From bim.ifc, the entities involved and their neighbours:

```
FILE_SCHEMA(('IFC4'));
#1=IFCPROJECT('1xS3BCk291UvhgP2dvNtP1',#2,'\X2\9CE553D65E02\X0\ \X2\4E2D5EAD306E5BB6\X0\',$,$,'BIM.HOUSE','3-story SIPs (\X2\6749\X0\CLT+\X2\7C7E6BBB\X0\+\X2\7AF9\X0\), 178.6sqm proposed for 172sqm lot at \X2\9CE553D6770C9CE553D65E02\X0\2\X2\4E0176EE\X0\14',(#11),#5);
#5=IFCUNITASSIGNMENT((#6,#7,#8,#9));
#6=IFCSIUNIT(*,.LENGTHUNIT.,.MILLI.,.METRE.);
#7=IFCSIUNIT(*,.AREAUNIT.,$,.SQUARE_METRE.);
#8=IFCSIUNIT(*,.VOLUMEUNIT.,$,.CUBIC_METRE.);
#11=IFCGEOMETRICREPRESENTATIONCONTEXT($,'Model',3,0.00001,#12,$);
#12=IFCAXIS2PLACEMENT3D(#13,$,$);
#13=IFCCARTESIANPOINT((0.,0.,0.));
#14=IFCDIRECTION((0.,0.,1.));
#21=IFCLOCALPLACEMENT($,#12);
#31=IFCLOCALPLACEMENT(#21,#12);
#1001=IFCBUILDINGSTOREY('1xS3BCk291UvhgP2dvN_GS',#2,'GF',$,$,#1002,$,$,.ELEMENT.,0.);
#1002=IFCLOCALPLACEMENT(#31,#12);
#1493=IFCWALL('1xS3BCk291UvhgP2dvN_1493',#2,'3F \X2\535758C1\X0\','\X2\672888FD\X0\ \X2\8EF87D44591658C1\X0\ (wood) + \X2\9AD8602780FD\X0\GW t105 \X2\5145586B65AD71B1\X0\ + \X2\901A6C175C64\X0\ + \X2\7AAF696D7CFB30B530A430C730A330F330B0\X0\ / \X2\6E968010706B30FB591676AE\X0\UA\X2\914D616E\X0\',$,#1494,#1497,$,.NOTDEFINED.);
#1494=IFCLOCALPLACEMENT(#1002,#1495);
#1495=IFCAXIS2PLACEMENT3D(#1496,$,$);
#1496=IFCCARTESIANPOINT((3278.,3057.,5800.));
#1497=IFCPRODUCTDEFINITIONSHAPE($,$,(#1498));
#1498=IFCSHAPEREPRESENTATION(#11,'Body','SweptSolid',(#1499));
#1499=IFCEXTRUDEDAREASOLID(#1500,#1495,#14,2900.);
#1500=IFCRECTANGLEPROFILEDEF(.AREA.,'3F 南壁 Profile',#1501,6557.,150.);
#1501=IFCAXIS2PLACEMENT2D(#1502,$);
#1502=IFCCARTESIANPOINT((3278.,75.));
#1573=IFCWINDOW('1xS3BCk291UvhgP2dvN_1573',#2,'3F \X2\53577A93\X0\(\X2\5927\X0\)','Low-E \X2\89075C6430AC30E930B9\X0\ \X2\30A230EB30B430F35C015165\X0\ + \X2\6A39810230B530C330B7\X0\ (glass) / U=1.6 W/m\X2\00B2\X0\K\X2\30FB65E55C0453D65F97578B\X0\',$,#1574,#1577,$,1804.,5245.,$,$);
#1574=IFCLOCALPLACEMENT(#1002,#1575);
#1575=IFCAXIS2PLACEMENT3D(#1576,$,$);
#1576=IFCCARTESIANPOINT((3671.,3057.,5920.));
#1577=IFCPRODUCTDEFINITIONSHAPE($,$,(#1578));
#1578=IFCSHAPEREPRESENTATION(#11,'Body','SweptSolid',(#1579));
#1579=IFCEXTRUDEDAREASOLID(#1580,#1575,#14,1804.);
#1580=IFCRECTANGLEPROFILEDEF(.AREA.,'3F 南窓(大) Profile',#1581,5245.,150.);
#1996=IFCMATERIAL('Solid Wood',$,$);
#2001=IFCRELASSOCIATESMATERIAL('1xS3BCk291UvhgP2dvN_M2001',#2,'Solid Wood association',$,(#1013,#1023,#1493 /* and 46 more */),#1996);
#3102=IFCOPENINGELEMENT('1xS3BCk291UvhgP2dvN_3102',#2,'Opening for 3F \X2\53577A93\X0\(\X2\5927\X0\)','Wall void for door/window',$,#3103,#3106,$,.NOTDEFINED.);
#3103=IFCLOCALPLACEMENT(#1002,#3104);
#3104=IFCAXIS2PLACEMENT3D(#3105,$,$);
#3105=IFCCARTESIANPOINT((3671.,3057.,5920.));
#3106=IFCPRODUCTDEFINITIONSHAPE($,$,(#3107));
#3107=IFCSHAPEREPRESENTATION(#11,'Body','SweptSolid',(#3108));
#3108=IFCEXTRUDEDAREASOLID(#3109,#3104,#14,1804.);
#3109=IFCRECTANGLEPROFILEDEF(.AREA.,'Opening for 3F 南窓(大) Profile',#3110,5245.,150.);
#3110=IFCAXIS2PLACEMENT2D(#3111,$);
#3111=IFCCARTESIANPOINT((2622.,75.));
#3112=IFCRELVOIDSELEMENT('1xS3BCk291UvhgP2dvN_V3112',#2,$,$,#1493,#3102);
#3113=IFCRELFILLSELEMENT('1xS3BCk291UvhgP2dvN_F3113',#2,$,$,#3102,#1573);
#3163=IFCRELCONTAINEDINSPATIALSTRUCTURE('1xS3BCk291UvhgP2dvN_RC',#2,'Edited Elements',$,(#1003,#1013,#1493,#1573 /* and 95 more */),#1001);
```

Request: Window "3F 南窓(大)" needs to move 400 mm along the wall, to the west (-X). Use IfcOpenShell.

```python
import ifcopenshell
import ifcopenshell.api.geometry
import ifcopenshell.util.placement
import ifcopenshell.util.unit

model = ifcopenshell.open("bim.ifc")
unit_scale = ifcopenshell.util.unit.calculate_unit_scale(model)

window = model.by_guid("1xS3BCk291UvhgP2dvN_1573")
opening = window.FillsVoids[0].RelatingOpeningElement
wall = opening.VoidsElements[0].RelatingBuildingElement

wall_matrix = ifcopenshell.util.placement.get_local_placement(wall.ObjectPlacement)
shift = wall_matrix[:3, 0] * -0.4 / unit_scale
before = ifcopenshell.util.placement.get_local_placement(window.ObjectPlacement)[:3, 3].copy()

# The window is not placed relative to its opening, so move both.
for product in (opening, window):
    matrix = ifcopenshell.util.placement.get_local_placement(product.ObjectPlacement)
    matrix[:3, 3] += shift
    ifcopenshell.api.geometry.edit_object_placement(model, product=product, matrix=matrix, is_si=False)

after = ifcopenshell.util.placement.get_local_placement(window.ObjectPlacement)[:3, 3]
print("window moved by", (after - before).round(3) + 0.0)

model.write("bim-out.ifc")
```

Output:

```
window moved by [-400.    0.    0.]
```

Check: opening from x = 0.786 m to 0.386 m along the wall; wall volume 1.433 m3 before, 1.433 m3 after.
